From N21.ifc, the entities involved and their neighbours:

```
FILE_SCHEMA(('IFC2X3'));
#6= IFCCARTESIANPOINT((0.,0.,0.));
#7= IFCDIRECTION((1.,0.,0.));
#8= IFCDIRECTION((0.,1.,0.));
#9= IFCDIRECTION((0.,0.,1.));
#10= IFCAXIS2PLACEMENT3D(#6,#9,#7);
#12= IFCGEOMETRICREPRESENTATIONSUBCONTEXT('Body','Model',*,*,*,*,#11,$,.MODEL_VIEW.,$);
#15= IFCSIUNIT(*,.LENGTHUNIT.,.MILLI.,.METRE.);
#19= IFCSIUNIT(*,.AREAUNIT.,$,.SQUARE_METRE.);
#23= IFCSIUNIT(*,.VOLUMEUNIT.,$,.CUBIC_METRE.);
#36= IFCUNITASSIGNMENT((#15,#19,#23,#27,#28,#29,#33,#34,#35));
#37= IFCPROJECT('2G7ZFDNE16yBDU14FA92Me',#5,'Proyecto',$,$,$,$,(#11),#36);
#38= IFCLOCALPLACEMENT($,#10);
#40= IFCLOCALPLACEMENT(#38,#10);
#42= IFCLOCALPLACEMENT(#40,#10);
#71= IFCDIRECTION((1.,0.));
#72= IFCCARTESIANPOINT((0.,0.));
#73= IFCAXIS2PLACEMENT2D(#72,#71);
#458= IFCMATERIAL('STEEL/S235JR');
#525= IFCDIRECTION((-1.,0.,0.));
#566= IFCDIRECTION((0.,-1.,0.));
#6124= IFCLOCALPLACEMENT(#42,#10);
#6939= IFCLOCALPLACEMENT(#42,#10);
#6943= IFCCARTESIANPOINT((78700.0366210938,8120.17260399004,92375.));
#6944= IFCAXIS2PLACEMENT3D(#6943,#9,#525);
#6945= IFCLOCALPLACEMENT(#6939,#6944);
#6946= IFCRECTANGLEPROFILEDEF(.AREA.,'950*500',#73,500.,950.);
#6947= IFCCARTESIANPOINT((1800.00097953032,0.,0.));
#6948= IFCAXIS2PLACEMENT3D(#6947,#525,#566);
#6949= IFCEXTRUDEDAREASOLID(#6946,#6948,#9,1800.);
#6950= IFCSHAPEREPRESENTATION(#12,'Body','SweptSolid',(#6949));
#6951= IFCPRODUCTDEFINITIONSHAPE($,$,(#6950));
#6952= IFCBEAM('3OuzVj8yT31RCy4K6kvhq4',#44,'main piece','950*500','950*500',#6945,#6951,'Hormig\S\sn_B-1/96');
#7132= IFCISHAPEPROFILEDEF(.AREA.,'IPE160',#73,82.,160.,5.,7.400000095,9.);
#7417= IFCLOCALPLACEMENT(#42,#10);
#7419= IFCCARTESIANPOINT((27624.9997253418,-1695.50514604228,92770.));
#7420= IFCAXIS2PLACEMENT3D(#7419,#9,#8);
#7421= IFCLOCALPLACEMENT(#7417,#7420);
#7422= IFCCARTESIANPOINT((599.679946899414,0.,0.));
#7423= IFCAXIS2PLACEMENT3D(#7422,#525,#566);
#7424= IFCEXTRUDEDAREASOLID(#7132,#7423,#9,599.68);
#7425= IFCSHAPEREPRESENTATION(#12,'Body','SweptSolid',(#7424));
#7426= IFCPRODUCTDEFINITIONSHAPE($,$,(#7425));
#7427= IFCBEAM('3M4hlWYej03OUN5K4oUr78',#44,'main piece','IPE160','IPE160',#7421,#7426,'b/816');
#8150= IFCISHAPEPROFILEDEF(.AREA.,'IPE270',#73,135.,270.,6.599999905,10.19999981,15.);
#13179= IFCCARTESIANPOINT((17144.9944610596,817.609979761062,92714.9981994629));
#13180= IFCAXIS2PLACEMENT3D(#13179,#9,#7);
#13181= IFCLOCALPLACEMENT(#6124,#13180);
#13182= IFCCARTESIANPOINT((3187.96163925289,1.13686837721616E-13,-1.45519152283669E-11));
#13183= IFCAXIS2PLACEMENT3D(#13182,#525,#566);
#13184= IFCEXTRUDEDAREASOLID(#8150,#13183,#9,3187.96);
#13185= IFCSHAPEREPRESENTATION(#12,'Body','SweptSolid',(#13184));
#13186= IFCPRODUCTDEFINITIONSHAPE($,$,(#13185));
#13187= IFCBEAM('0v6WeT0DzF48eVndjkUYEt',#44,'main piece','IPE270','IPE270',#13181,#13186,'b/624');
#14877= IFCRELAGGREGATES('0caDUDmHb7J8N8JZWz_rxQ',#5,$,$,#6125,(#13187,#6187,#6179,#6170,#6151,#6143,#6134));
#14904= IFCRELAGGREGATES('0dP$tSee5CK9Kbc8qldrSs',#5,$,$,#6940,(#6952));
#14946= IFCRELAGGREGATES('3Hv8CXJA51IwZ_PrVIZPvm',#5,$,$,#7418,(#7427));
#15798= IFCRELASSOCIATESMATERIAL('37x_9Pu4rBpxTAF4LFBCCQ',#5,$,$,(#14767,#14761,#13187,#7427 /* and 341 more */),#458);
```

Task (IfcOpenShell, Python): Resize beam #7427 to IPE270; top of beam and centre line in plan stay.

```python
import ifcopenshell
import ifcopenshell.util.element
import ifcopenshell.util.representation

model = ifcopenshell.open("N21.ifc")

member = model.by_guid("3M4hlWYej03OUN5K4oUr78")
source = next(p for p in model.by_type("IfcIShapeProfileDef") if p.ProfileName == "IPE270")

body = ifcopenshell.util.representation.get_representation(member, "Model", "Body")
solid = body.Items[0]
old_profile = solid.SweptArea

# Copy the section's sizes but keep this member's own profile position.
profile = ifcopenshell.util.element.copy(model, source)
# Profiles are centred, so shift by half the change in depth to hold the top.
shift = (old_profile.OverallDepth - profile.OverallDepth) / 2
x, y = old_profile.Position.Location.Coordinates
up = (0.0, 1.0)  # upwards, in the solid's own plane
location = model.createIfcCartesianPoint((x + up[0] * shift, y + up[1] * shift))
profile.Position = model.createIfcAxis2Placement2D(location, old_profile.Position.RefDirection)
solid.SweptArea = profile
if not model.get_total_inverses(old_profile):
    ifcopenshell.util.element.remove_deep2(model, old_profile)
member.Description = member.Description.replace("IPE160", "IPE270")
member.ObjectType = member.ObjectType.replace("IPE160", "IPE270")

print(solid.SweptArea)

model.write("N21_edited.ifc")
```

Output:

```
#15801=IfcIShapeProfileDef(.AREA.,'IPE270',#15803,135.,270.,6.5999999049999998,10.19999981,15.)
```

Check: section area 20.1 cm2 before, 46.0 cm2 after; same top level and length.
